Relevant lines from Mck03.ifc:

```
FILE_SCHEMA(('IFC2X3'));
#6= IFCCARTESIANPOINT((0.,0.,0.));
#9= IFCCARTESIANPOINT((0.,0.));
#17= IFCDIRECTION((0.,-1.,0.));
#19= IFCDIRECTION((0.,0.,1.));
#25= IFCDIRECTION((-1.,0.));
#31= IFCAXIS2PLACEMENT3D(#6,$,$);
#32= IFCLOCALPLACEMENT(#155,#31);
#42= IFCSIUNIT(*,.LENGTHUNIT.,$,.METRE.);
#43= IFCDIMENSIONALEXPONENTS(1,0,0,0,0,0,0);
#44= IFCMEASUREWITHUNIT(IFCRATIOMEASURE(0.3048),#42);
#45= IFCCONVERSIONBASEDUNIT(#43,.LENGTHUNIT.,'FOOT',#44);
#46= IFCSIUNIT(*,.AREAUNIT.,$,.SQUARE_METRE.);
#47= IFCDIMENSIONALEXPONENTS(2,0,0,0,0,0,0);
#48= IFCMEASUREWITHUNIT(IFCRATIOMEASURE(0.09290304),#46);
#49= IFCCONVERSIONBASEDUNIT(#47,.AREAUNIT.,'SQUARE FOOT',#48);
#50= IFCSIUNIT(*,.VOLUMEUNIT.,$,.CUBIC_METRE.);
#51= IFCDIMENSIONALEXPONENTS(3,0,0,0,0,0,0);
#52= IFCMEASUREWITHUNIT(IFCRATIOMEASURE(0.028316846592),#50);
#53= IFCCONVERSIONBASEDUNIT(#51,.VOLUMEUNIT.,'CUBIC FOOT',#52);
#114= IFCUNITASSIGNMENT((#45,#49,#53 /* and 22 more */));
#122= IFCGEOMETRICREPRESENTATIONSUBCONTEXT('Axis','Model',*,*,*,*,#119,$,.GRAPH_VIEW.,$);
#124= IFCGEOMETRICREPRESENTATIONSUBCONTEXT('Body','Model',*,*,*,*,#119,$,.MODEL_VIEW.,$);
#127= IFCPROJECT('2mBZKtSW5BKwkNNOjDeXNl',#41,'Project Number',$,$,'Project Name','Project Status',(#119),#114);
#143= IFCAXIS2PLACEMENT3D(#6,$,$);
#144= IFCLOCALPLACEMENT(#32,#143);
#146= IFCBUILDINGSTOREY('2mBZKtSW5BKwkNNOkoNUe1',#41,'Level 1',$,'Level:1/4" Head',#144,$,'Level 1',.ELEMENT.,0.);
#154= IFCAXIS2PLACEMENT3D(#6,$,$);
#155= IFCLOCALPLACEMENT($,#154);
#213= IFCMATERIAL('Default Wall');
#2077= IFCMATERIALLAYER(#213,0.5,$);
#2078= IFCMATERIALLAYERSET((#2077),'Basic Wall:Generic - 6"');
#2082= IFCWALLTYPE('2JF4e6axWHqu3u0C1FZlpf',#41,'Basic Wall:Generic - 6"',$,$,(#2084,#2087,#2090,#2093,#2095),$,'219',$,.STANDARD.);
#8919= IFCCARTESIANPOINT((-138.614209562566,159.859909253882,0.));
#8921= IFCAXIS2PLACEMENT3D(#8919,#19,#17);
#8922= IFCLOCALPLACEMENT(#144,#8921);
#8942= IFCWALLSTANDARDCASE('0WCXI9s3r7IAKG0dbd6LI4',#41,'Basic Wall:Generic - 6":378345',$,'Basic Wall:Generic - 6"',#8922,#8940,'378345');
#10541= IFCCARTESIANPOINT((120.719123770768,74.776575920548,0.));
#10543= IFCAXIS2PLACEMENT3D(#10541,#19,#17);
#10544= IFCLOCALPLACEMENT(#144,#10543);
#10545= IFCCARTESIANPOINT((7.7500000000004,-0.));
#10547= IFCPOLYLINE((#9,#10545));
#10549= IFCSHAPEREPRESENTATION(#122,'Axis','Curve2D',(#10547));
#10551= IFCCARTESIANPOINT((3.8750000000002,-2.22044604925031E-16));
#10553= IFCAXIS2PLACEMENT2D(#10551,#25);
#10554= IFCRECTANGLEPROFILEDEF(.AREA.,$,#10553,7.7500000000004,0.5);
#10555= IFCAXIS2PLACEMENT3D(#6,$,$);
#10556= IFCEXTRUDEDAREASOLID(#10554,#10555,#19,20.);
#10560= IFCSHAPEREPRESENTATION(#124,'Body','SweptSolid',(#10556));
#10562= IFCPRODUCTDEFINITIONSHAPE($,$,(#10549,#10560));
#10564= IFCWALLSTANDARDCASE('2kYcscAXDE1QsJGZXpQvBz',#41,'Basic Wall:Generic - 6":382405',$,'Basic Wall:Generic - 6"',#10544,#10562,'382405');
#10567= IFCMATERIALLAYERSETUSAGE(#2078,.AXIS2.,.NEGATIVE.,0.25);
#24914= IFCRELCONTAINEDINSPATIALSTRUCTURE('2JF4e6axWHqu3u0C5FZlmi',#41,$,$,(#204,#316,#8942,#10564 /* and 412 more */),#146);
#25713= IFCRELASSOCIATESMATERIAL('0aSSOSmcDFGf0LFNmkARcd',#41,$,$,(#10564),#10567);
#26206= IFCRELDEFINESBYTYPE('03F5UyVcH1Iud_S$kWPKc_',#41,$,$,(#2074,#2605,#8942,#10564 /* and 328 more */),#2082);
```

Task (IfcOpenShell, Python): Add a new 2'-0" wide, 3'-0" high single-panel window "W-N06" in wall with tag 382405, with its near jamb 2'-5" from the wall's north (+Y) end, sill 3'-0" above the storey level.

```python
import numpy as np
import ifcopenshell
import ifcopenshell.api.feature
import ifcopenshell.api.geometry
import ifcopenshell.api.root
import ifcopenshell.api.spatial
import ifcopenshell.api.type
import ifcopenshell.geom
import ifcopenshell.util.element
import ifcopenshell.util.placement
import ifcopenshell.util.representation
import ifcopenshell.util.shape
import ifcopenshell.util.unit

model = ifcopenshell.open("Mck03.ifc")
unit_scale = ifcopenshell.util.unit.calculate_unit_scale(model)
settings = ifcopenshell.geom.settings()


def volume(element):
    """Net volume in cubic metres, openings subtracted."""
    shape = ifcopenshell.geom.create_shape(settings, element)
    return ifcopenshell.util.shape.get_volume(shape.geometry)


wall = model.by_id(10564)
storey = ifcopenshell.util.element.get_container(wall, ifc_class="IfcBuildingStorey")
context = ifcopenshell.util.representation.get_context(model, "Model", "Body", "MODEL_VIEW")
before = volume(wall)

width, height, from_end, sill = 0.6096, 0.9144, 0.7366, 0.9144  # metres

# The wall runs along its own X axis, and the end named is its -X end.
wall_shape = ifcopenshell.geom.create_shape(settings, wall)
x, y, z = ifcopenshell.util.shape.get_vertices(wall_shape.geometry).T
start = x.min() + from_end
face, thickness = float(y.min()), float(y.max() - y.min())
wall_matrix = ifcopenshell.util.placement.get_local_placement(wall.ObjectPlacement)
level = ifcopenshell.util.placement.get_local_placement(storey.ObjectPlacement)[2, 3]


def in_wall(x, y):
    """Placement at x, y metres in the wall's axes, at sill height."""
    matrix = wall_matrix.copy()
    matrix[:, 3] = wall_matrix @ np.array([x / unit_scale, y / unit_scale, 0.0, 1.0])
    matrix[2, 3] = level + sill / unit_scale
    return matrix


# Opening: a box that overshoots both wall faces by 50 mm.
opening = ifcopenshell.api.root.create_entity(model, ifc_class="IfcOpeningElement")
box = ifcopenshell.api.geometry.add_wall_representation(
    model, context=context, length=width, height=height, thickness=thickness + 0.1
)
ifcopenshell.api.geometry.assign_representation(model, product=opening, representation=box)
ifcopenshell.api.geometry.edit_object_placement(model, product=opening, matrix=in_wall(start, face - 0.05), is_si=False)
ifcopenshell.api.feature.add_feature(model, feature=opening, element=wall)

window = ifcopenshell.api.root.create_entity(model, ifc_class="IfcWindow", name="W-N06")
window.OverallWidth, window.OverallHeight = width / unit_scale, height / unit_scale
body = ifcopenshell.api.geometry.add_window_representation(
    model,
    context=context,
    overall_width=window.OverallWidth,
    overall_height=window.OverallHeight,
    partition_type="SINGLE_PANEL",
)
ifcopenshell.api.geometry.assign_representation(model, product=window, representation=body)
ifcopenshell.api.spatial.assign_container(model, products=[window], relating_structure=storey)
fills = ifcopenshell.api.feature.add_filling(model, opening=opening, element=window)
fills.OwnerHistory = window.OwnerHistory  # required in IFC2X3

# IFC2X3 keeps the operation on the window style.
style = ifcopenshell.api.root.create_entity(model, ifc_class="IfcWindowStyle", name="W-N06")
style.OperationType, style.ConstructionType = "SINGLE_PANEL", "NOTDEFINED"
style.ParameterTakesPrecedence = style.Sizeable = False
ifcopenshell.api.type.assign_type(model, related_objects=[window], relating_type=style)

# Centre the window in the wall's thickness.
ifcopenshell.api.geometry.edit_object_placement(model, product=window, matrix=in_wall(start, face), is_si=False)
window_shape = ifcopenshell.geom.create_shape(settings, window)
depth = ifcopenshell.util.shape.get_vertices(window_shape.geometry)[:, 1]
offset = face + thickness / 2 - (depth.min() + depth.max()) / 2
ifcopenshell.api.geometry.edit_object_placement(model, product=window, matrix=in_wall(start, offset), is_si=False)

after = volume(wall)

print(f"wall volume {before:.3f} -> {after:.3f} m3")

model.write("Mck03_updated.ifc")
```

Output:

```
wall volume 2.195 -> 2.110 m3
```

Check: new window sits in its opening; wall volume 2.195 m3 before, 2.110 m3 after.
